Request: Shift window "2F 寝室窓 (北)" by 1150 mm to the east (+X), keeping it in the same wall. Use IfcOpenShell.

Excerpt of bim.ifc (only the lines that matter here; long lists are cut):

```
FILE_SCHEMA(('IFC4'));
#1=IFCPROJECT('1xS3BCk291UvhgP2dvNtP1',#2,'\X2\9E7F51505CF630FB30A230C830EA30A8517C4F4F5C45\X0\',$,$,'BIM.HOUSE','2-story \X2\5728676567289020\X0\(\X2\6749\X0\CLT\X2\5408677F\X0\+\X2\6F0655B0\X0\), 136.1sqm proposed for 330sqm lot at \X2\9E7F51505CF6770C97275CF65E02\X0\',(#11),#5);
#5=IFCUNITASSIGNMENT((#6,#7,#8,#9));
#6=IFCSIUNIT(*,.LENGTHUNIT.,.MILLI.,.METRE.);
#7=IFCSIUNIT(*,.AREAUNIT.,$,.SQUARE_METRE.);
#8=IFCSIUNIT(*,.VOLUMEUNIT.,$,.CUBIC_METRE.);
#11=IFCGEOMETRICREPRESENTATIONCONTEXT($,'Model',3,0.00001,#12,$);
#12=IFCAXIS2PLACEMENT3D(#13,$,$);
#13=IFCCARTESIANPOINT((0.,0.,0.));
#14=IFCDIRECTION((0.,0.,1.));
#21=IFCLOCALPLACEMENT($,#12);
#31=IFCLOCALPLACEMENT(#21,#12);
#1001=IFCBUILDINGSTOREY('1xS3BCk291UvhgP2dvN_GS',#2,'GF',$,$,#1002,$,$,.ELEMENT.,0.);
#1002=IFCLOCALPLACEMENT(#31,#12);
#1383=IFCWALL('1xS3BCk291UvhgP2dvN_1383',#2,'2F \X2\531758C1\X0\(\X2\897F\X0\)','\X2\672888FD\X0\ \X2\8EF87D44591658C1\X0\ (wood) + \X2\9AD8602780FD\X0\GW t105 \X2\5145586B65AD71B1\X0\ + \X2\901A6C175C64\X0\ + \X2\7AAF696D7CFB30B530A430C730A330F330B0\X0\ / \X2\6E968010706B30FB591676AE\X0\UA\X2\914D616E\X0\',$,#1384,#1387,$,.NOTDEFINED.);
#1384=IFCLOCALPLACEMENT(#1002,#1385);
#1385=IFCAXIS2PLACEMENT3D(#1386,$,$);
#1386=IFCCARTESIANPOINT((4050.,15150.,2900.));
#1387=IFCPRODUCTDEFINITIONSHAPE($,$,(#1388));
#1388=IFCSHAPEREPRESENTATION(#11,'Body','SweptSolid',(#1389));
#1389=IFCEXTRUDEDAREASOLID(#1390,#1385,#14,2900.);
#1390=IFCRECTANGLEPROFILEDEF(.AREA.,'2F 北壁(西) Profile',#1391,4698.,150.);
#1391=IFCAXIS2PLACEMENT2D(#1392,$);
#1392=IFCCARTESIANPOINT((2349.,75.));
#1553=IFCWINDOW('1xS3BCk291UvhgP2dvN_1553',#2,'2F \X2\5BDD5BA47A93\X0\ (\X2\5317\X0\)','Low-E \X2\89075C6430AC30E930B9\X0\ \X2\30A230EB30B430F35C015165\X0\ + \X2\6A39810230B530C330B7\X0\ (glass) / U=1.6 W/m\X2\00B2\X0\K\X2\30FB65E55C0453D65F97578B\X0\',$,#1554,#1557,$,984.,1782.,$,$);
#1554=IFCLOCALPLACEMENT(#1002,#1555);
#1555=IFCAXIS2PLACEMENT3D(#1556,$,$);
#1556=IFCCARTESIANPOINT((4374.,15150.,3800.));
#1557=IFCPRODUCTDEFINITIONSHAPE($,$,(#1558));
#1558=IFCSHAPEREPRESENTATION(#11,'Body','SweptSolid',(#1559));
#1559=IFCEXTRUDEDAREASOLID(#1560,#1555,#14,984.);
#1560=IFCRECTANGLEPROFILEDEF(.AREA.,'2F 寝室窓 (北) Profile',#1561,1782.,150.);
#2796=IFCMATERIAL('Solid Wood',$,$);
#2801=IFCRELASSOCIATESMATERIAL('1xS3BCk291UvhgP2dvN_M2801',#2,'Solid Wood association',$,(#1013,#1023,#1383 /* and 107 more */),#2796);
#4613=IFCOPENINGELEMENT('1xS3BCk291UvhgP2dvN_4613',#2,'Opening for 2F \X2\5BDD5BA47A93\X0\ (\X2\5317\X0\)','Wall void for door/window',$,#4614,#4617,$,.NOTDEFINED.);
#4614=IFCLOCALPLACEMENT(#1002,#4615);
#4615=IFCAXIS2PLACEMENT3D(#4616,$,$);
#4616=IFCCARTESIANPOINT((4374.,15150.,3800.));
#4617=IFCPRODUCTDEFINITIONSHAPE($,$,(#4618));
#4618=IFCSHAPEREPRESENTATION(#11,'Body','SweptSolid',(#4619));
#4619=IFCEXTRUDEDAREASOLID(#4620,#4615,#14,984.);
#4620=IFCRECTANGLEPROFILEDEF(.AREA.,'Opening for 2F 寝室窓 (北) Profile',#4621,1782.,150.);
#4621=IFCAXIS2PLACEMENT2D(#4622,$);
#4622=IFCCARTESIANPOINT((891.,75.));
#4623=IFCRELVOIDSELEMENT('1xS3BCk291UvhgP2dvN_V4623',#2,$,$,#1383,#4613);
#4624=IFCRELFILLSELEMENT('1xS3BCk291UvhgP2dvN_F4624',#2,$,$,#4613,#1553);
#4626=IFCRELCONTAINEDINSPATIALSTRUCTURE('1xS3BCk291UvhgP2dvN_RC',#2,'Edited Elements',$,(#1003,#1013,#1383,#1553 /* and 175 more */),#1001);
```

```python
import ifcopenshell
import ifcopenshell.api.geometry
import ifcopenshell.util.placement

model = ifcopenshell.open("bim.ifc")

window = model.by_id(1553)
opening = window.FillsVoids[0].RelatingOpeningElement
wall = opening.VoidsElements[0].RelatingBuildingElement

wall_matrix = ifcopenshell.util.placement.get_local_placement(wall.ObjectPlacement)
shift = wall_matrix[:3, 0] * 1150.0
before = ifcopenshell.util.placement.get_local_placement(window.ObjectPlacement)[:3, 3].copy()

# The window is not placed relative to its opening, so move both.
for product in (opening, window):
    matrix = ifcopenshell.util.placement.get_local_placement(product.ObjectPlacement)
    matrix[:3, 3] += shift
    ifcopenshell.api.geometry.edit_object_placement(model, product=product, matrix=matrix, is_si=False)

after = ifcopenshell.util.placement.get_local_placement(window.ObjectPlacement)[:3, 3]
print("window moved by", (after - before).round(3) + 0.0)

model.write("bim_updated.ifc")
```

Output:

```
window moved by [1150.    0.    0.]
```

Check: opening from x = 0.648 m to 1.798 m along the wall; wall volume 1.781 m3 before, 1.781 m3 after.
